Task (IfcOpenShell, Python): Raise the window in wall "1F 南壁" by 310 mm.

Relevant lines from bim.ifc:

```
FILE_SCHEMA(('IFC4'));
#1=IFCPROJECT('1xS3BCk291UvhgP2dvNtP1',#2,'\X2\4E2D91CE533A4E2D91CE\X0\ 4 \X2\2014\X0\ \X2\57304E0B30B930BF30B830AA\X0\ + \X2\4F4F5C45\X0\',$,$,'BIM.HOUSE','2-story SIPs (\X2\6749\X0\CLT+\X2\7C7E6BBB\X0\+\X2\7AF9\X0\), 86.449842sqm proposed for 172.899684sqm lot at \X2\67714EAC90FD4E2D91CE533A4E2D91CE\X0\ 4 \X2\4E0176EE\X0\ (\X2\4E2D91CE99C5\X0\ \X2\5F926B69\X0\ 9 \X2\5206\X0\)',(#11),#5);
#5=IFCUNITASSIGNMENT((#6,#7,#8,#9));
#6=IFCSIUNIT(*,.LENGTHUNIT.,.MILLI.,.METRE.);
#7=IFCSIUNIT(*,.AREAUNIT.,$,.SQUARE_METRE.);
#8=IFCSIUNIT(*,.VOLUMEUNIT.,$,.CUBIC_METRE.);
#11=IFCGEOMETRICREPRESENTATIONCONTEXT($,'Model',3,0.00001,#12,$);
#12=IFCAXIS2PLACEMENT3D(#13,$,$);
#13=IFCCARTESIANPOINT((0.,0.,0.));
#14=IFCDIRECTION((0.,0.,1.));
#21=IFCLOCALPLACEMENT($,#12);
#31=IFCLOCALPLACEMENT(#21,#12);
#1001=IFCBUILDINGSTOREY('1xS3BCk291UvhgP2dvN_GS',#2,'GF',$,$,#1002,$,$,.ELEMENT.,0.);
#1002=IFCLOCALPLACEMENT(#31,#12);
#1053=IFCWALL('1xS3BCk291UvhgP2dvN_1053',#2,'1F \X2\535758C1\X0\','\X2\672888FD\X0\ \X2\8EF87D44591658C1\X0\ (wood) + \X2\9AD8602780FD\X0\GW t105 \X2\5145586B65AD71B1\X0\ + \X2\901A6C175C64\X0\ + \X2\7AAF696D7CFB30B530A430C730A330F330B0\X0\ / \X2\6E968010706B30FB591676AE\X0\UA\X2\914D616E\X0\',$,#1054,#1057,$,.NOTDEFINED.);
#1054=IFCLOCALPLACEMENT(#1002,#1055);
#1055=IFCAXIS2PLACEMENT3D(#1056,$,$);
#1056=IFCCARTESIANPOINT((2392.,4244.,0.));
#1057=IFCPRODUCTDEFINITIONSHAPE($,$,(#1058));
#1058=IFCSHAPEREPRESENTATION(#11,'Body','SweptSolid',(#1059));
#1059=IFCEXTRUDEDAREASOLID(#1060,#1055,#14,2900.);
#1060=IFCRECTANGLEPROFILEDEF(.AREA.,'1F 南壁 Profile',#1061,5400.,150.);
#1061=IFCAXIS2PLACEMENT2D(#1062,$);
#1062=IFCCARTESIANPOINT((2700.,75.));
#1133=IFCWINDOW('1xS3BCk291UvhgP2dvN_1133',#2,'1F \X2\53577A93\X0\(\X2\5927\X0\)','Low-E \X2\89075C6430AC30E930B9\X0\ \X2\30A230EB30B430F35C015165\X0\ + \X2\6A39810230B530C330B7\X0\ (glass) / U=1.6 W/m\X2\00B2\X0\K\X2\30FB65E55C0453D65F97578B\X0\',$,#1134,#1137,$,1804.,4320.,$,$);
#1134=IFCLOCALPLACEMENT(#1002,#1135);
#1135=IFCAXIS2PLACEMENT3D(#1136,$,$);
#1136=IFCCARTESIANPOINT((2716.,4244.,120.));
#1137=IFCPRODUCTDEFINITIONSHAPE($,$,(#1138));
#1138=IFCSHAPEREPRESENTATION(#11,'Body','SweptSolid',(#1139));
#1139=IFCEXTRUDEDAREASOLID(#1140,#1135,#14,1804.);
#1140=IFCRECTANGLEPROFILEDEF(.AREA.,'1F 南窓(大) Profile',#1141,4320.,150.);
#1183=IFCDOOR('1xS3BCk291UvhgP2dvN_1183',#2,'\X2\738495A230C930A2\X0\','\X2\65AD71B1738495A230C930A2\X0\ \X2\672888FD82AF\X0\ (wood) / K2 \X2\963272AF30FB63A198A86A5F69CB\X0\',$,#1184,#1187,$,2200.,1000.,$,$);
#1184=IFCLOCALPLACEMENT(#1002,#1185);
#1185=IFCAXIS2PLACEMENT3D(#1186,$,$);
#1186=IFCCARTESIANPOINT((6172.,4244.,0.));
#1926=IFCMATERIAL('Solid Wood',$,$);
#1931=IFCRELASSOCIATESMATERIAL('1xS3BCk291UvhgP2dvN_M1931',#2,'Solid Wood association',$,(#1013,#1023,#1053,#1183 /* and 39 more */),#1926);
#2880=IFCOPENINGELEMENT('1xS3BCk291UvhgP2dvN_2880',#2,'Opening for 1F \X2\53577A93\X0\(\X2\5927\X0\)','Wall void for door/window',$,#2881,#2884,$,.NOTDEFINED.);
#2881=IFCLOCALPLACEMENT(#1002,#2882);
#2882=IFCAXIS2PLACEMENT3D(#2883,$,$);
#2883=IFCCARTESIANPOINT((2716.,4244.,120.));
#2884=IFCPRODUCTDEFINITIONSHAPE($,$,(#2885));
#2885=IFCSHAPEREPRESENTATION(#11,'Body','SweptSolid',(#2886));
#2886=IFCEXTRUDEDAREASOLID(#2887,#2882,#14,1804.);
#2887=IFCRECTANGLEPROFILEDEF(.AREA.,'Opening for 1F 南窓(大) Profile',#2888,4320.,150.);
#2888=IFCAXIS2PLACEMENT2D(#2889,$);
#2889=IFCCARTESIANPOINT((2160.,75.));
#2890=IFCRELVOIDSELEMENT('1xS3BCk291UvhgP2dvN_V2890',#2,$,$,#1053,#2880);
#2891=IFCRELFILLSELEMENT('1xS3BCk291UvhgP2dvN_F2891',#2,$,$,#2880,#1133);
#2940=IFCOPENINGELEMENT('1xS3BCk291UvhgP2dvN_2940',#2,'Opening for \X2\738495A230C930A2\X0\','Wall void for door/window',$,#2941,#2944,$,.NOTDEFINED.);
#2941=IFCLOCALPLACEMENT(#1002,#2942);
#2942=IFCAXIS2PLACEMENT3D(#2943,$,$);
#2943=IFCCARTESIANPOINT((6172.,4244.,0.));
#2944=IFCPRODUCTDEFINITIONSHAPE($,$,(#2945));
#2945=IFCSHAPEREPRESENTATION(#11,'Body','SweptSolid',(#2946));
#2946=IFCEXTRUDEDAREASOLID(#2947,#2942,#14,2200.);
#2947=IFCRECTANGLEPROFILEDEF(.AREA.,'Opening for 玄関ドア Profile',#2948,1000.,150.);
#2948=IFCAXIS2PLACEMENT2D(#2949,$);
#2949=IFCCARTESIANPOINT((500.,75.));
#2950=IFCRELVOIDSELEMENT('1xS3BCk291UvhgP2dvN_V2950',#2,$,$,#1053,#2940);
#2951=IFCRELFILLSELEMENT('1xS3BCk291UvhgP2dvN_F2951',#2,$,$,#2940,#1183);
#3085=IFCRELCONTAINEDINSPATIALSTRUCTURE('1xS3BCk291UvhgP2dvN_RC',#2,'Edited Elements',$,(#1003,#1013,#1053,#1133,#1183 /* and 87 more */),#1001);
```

```python
import numpy as np
import ifcopenshell
import ifcopenshell.api.geometry
import ifcopenshell.util.placement
import ifcopenshell.util.unit

model = ifcopenshell.open("bim.ifc")
unit_scale = ifcopenshell.util.unit.calculate_unit_scale(model)

window = model.by_guid("1xS3BCk291UvhgP2dvN_1133")
opening = window.FillsVoids[0].RelatingOpeningElement
dz = 310.0

shift = np.array([0.0, 0.0, dz])
# The window is not placed relative to its opening, so move both.
for product in (opening, window):
    matrix = ifcopenshell.util.placement.get_local_placement(product.ObjectPlacement)
    matrix[:3, 3] += shift
    ifcopenshell.api.geometry.edit_object_placement(model, product=product, matrix=matrix, is_si=False)

print(f"moved by {dz * unit_scale:+.3f} m")

model.write("bim_edited.ifc")
```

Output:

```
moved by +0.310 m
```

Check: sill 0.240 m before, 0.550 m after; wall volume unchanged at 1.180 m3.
